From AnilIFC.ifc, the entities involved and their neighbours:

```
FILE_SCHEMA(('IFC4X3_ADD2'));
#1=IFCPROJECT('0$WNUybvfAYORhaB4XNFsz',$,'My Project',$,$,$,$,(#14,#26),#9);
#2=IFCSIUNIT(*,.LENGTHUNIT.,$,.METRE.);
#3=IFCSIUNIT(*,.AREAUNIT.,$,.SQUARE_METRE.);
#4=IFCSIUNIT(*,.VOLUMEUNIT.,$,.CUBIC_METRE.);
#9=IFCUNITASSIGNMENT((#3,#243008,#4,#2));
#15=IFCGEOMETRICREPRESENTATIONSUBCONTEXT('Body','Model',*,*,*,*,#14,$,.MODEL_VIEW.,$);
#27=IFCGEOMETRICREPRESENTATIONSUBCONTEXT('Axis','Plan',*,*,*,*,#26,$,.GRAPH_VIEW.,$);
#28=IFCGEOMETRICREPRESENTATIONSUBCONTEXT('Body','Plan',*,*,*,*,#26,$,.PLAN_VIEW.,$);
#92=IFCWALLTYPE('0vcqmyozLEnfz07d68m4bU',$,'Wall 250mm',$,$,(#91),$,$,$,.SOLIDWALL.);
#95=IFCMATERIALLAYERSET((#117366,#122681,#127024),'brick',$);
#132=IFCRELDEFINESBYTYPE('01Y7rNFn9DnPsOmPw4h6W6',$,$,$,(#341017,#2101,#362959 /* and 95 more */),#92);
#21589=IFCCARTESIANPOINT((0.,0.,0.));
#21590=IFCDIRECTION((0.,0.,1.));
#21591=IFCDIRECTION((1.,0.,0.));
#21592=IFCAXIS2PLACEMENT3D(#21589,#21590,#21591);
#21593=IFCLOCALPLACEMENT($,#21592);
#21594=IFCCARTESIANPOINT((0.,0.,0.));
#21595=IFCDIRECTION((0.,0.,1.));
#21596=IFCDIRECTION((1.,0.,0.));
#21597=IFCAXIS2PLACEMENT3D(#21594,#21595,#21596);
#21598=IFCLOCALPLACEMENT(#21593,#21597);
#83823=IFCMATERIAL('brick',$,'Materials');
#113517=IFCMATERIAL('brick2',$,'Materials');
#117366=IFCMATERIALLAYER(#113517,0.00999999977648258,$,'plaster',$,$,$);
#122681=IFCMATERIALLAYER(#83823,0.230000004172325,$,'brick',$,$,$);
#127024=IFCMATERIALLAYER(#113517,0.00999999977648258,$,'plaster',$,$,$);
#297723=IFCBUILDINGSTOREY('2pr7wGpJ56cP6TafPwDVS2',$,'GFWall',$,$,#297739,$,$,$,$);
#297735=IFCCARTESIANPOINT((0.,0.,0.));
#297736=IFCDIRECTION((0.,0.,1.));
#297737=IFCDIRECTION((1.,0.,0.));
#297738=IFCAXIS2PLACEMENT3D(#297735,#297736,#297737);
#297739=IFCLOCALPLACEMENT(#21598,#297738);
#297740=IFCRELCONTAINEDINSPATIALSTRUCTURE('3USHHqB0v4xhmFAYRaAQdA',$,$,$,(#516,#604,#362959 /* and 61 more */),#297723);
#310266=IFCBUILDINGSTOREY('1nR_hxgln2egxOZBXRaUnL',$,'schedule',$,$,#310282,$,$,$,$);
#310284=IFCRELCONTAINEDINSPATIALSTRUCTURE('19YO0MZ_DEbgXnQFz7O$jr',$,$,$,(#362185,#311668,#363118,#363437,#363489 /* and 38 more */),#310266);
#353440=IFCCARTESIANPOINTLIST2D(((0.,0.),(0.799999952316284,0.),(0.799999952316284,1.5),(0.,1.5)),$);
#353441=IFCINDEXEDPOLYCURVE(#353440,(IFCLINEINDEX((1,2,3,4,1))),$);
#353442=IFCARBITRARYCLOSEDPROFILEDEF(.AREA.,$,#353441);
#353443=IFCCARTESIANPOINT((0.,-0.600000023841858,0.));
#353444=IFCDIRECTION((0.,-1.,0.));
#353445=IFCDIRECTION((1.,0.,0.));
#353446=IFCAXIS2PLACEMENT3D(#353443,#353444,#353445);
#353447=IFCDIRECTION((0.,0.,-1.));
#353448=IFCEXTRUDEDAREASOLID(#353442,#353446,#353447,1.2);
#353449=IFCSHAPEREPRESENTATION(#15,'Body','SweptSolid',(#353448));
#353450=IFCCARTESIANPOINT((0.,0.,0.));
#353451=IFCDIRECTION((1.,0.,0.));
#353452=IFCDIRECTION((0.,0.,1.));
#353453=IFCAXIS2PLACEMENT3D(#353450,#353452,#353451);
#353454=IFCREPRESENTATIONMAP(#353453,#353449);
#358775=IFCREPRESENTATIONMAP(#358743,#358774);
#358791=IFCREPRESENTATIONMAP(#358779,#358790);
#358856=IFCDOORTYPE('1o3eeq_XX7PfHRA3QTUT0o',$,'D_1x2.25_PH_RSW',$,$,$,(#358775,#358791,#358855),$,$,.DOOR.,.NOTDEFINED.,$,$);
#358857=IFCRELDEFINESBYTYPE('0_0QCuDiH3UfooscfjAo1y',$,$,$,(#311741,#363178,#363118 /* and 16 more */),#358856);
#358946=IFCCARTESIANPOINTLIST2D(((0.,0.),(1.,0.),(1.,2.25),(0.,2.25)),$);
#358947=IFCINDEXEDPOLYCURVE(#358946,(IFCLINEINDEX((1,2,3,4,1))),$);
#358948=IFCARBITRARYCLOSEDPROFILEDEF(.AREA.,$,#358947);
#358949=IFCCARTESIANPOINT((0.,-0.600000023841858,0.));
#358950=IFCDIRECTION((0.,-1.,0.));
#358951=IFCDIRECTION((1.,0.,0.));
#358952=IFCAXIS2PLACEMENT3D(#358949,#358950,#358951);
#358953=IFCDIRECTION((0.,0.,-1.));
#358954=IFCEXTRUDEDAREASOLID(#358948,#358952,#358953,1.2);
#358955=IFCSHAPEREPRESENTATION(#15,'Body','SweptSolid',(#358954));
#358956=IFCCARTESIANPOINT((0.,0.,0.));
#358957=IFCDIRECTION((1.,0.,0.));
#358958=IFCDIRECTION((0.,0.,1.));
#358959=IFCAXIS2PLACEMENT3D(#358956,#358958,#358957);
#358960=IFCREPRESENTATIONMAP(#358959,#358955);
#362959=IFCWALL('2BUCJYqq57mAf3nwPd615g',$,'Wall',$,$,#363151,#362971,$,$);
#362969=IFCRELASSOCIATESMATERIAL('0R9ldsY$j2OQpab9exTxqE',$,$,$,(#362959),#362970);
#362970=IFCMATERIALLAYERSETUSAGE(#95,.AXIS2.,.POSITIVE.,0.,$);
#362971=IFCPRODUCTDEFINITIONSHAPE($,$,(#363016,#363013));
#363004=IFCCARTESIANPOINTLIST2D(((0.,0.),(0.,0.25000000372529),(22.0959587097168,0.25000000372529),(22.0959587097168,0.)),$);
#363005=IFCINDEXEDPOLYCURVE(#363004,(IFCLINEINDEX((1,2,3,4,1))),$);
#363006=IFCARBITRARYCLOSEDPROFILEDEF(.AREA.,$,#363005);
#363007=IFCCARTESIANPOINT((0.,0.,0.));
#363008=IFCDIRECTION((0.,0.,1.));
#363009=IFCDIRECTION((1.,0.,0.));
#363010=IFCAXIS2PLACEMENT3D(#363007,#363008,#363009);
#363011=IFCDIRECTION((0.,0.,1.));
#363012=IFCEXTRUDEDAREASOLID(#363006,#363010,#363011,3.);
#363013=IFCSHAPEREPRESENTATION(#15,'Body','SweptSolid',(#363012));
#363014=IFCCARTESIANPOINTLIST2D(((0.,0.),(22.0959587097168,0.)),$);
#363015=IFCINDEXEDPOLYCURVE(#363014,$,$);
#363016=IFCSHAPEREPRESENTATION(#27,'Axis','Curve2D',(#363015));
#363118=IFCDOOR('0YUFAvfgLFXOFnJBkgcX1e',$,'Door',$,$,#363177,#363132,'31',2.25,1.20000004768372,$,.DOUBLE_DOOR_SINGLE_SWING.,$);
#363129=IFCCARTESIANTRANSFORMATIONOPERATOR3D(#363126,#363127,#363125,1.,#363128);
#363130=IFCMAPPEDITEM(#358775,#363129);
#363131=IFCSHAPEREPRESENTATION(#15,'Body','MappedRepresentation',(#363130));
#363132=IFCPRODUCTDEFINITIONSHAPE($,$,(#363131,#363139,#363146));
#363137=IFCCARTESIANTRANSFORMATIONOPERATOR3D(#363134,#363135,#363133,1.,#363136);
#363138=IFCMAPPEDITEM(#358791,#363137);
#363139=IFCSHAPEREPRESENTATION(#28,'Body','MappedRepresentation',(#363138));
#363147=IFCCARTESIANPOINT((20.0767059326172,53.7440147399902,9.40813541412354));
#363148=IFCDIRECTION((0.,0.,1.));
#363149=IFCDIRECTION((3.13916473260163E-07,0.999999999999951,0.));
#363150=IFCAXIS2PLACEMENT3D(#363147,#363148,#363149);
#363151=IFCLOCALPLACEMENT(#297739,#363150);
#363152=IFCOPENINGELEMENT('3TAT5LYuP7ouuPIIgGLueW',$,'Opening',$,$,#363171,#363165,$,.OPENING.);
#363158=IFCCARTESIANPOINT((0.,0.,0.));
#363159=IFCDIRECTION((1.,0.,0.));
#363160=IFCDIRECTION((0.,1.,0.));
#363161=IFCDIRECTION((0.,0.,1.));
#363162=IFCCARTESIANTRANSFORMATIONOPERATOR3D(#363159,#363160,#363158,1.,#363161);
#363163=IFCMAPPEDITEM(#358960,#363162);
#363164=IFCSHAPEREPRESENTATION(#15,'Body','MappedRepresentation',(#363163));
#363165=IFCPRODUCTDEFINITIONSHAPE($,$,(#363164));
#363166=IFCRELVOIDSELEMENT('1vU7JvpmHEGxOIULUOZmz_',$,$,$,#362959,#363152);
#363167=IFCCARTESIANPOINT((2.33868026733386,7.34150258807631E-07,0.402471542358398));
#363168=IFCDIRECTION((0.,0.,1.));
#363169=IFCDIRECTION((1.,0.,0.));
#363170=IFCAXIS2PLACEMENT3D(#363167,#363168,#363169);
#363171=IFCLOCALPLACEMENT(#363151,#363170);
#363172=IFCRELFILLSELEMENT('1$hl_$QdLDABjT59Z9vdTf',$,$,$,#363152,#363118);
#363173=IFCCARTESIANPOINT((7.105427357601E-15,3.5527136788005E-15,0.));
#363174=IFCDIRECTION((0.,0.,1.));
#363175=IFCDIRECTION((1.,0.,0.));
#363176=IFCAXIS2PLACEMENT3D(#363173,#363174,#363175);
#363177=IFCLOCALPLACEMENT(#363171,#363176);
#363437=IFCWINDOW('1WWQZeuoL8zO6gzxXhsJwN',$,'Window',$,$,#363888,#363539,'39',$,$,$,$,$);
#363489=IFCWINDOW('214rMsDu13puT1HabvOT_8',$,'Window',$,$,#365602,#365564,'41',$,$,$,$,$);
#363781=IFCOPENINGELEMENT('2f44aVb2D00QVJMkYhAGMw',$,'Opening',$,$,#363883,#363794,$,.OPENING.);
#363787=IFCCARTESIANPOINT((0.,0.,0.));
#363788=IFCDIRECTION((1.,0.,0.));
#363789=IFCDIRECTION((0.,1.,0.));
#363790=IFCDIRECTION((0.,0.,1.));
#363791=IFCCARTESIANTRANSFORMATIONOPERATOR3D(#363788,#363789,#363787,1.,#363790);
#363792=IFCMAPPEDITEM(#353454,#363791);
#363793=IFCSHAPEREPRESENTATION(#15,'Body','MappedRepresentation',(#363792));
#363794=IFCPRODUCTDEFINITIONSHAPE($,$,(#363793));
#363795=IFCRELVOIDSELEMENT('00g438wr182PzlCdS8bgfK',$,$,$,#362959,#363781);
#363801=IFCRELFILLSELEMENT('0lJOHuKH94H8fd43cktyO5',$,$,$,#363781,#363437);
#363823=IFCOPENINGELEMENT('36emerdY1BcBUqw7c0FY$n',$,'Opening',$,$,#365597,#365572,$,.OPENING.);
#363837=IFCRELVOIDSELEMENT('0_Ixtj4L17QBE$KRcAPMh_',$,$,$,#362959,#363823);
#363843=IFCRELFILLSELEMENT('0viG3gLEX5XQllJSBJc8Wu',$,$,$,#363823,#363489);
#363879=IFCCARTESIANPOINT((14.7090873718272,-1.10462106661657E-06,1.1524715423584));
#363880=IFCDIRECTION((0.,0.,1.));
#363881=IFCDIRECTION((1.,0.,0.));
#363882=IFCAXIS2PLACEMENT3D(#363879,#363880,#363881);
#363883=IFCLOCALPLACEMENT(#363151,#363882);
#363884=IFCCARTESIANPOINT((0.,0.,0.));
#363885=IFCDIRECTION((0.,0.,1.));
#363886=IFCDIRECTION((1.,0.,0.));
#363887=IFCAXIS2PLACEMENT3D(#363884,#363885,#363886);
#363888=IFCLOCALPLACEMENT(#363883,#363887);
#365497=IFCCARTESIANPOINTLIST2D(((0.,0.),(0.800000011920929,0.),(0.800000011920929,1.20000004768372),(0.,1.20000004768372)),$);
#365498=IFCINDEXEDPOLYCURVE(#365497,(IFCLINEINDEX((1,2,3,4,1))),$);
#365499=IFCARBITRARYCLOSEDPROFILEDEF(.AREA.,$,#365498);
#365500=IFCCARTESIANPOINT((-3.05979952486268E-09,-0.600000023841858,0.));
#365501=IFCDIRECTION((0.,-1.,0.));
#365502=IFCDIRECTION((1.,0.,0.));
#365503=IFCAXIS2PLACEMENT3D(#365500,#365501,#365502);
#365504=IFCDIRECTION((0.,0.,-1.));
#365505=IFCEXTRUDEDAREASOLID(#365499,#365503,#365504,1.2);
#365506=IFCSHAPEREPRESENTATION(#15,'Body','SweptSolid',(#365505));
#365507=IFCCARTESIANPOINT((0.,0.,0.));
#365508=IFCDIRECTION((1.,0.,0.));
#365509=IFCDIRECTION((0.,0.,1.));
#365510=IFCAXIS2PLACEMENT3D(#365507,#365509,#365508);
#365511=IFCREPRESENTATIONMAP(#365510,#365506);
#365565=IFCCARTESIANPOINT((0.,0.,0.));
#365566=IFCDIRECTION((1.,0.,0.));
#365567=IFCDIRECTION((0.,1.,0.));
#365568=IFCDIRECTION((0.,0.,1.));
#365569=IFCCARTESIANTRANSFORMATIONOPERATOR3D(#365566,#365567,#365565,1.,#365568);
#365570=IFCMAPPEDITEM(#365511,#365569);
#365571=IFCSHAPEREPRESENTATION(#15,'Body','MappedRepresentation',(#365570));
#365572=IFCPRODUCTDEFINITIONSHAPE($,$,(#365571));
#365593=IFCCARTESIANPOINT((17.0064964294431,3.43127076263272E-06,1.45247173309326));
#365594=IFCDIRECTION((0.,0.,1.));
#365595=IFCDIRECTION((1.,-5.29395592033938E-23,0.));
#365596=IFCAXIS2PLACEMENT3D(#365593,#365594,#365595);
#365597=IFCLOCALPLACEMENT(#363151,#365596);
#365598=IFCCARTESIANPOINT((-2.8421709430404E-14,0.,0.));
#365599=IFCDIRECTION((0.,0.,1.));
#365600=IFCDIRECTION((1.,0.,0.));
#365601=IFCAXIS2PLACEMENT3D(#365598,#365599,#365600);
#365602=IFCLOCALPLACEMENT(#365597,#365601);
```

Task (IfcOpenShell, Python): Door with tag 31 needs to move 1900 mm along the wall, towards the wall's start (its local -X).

```python
import ifcopenshell
import ifcopenshell.api.geometry
import ifcopenshell.util.placement

model = ifcopenshell.open("AnilIFC.ifc")

door = model.by_id(363118)
opening = door.FillsVoids[0].RelatingOpeningElement
wall = opening.VoidsElements[0].RelatingBuildingElement

wall_matrix = ifcopenshell.util.placement.get_local_placement(wall.ObjectPlacement)
shift = wall_matrix[:3, 0] * -1.9
before = ifcopenshell.util.placement.get_local_placement(door.ObjectPlacement)[:3, 3].copy()

# The door is placed relative to its opening, so it follows when the opening moves.
matrix = ifcopenshell.util.placement.get_local_placement(opening.ObjectPlacement)
matrix[:3, 3] += shift
ifcopenshell.api.geometry.edit_object_placement(
    model, product=opening, matrix=matrix, is_si=False, should_transform_children=True
)

after = ifcopenshell.util.placement.get_local_placement(door.ObjectPlacement)[:3, 3]
print("door moved by", (after - before).round(3) + 0.0)

model.write("AnilIFC_edited.ifc")
```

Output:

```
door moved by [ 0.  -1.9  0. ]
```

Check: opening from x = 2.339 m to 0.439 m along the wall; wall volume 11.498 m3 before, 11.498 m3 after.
